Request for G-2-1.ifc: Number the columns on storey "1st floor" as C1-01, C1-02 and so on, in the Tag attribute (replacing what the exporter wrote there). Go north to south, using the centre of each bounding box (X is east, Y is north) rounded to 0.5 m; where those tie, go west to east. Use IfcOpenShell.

First a look at what the model holds.

```python
import ifcopenshell
import ifcopenshell.util.element
import ifcopenshell.util.placement

model = ifcopenshell.open("G-2-1.ifc")
print(model.schema)
storey = next(s for s in model.by_type("IfcBuildingStorey") if s.Name == "1st floor")
columns = [e for e in ifcopenshell.util.element.get_decomposition(storey) if e.is_a("IfcColumn")]
for e in sorted(columns, key=lambda e: e.id()):
    origin = ifcopenshell.util.placement.get_local_placement(e.ObjectPlacement)[:3, 3]
    print(e.id(), e.Tag, e.Name, origin.round(2) + 0.0, sep=" | ")
```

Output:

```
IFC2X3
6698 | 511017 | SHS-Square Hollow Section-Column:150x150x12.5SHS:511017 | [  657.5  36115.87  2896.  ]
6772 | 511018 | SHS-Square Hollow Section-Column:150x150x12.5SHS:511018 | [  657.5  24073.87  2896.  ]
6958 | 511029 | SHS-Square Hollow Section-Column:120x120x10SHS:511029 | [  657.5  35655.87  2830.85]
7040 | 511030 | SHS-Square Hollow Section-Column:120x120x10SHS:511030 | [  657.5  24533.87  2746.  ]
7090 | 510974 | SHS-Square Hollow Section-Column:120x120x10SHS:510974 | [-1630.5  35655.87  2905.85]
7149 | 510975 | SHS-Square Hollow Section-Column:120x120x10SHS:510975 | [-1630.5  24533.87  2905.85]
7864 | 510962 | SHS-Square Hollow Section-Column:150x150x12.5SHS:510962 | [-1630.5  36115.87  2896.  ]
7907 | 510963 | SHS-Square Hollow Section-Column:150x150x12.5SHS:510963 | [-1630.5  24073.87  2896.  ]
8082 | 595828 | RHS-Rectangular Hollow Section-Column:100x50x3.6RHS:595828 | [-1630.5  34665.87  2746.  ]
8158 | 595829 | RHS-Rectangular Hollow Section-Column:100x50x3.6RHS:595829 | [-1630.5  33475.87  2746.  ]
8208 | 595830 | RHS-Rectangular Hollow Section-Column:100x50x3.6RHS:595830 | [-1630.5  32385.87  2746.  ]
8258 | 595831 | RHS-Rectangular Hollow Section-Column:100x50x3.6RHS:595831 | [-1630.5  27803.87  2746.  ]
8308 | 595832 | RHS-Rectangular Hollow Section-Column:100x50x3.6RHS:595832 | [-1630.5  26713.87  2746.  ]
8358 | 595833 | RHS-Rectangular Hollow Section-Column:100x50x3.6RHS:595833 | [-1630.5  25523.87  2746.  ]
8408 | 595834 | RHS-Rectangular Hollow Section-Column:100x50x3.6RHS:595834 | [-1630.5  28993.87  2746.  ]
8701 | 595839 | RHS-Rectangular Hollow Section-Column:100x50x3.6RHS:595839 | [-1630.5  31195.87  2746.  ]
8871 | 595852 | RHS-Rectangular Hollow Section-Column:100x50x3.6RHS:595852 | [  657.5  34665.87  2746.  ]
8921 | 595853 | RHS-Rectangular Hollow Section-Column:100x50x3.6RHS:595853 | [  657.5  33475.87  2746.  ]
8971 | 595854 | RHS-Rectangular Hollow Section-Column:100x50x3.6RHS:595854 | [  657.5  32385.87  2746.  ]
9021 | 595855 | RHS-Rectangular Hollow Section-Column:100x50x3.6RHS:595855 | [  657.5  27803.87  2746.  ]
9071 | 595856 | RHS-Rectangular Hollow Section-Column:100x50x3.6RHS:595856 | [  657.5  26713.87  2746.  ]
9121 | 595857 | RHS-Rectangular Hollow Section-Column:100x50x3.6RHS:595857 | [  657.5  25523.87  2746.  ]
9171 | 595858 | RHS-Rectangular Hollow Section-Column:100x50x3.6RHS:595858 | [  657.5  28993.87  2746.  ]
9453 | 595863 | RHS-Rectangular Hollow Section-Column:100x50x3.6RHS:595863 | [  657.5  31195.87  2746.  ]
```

```python
import ifcopenshell
import ifcopenshell.geom
import ifcopenshell.util.element
import ifcopenshell.util.shape

model = ifcopenshell.open("G-2-1.ifc")
settings = ifcopenshell.geom.settings()
settings.set("use-world-coords", True)


def centre(element):
    shape = ifcopenshell.geom.create_shape(settings, element)
    return ifcopenshell.util.shape.get_bbox_centroid(shape.geometry)


storey = next(s for s in model.by_type("IfcBuildingStorey") if s.Name == "1st floor")
columns = [e for e in ifcopenshell.util.element.get_decomposition(storey) if e.is_a("IfcColumn")]

# Insertion points can sit at a corner or the storey origin, so sort by the geometry (in metres).
centres = {e: centre(e) for e in columns}
columns.sort(key=lambda e: (-round(centres[e][1] / 0.5), centres[e][0]))

for i, e in enumerate(columns, start=1):
    number = f"C1-{i:02d}"
    e.Tag = number
    print(e.id(), number)

model.write("G-2-1-out.ifc")
```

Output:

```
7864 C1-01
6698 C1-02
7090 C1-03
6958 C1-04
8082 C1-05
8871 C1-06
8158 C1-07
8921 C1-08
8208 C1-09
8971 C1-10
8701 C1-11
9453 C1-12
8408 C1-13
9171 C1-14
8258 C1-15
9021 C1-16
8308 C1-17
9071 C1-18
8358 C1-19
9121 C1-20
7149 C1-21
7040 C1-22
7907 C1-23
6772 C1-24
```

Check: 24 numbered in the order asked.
